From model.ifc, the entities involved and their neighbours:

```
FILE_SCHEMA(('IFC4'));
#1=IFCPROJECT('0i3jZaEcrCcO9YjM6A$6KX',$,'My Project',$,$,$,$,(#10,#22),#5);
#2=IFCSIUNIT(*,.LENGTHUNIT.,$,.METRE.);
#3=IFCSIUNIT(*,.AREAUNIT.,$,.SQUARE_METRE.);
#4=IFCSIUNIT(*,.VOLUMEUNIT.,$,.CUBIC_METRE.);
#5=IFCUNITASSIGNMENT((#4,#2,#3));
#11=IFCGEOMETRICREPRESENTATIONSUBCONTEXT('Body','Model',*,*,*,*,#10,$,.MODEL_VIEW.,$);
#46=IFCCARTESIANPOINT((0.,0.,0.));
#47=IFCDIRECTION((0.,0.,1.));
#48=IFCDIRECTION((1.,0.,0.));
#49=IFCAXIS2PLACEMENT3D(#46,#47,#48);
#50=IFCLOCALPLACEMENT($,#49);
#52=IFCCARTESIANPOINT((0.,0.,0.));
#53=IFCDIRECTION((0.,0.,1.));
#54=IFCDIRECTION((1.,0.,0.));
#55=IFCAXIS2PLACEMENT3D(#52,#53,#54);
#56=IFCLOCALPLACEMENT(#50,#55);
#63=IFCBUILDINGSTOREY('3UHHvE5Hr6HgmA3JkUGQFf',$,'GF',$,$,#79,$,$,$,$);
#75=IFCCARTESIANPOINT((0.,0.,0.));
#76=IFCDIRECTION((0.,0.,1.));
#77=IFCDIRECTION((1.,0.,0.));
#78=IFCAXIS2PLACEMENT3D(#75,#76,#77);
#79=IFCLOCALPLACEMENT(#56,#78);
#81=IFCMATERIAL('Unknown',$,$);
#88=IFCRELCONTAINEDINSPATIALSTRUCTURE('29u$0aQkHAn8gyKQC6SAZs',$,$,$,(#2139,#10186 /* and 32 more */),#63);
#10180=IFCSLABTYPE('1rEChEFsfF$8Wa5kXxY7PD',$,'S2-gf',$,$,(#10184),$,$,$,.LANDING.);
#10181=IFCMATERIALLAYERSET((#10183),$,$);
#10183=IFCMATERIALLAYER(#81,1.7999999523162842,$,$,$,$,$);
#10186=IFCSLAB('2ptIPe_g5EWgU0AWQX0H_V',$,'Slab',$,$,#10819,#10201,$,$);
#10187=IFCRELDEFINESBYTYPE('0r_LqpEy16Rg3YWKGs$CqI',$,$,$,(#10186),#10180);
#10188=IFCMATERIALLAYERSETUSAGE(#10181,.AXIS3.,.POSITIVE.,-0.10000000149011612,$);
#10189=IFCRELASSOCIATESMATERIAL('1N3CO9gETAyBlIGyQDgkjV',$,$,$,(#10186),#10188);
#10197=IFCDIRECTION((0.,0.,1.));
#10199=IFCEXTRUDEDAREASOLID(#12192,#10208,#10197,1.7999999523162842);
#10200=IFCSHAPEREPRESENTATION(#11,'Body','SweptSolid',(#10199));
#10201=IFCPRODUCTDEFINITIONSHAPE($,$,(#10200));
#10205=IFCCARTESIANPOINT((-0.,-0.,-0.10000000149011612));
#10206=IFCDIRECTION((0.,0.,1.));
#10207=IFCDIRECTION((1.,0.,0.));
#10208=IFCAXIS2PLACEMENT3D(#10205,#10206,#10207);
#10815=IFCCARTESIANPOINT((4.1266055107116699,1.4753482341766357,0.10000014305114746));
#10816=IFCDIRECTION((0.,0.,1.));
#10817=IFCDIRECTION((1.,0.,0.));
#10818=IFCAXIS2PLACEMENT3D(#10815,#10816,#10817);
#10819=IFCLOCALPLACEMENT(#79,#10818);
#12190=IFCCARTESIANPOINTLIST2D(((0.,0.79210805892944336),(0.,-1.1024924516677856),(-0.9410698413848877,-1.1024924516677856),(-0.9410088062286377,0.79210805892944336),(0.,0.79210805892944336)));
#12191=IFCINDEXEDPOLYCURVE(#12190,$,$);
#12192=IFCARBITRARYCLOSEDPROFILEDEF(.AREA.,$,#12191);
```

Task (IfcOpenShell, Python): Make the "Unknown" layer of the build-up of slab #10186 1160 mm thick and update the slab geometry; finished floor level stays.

```python
import ifcopenshell
import ifcopenshell.util.element
import ifcopenshell.util.representation
import ifcopenshell.util.unit

model = ifcopenshell.open("model.ifc")
unit_scale = ifcopenshell.util.unit.calculate_unit_scale(model)

layer_set = model.by_id(10181)
layer = next(l for l in layer_set.MaterialLayers if l.Material and l.Material.Name == "Unknown")
change = 1.16 / unit_scale - layer.LayerThickness
layer.LayerThickness += change

# Geometry does not follow the layer set by itself.
slabs = [e for e in ifcopenshell.util.element.get_elements_by_material(model, layer_set) if e.is_a("IfcSlab")]
for slab in sorted(slabs, key=lambda e: e.id()):
    body = ifcopenshell.util.representation.get_representation(slab, "Model", "Body")
    solid = body.Items[0]
    old_depth = solid.Depth
    solid.Depth += change
    # Extruded upwards: lower the start of the extrusion so the top stays.
    x, y, z = solid.Position.Location.Coordinates
    solid.Position.Location = model.createIfcCartesianPoint((x, y, z - change))
    print(slab.id(), f"{old_depth:g} -> {solid.Depth:g}")

# The layers are counted up from the underside, which has moved.
for usage in {ifcopenshell.util.element.get_material(slab) for slab in slabs}:
    usage.OffsetFromReferenceLine -= change

model.write("model_rev.ifc")
```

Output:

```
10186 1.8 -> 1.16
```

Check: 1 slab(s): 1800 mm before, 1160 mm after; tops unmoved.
